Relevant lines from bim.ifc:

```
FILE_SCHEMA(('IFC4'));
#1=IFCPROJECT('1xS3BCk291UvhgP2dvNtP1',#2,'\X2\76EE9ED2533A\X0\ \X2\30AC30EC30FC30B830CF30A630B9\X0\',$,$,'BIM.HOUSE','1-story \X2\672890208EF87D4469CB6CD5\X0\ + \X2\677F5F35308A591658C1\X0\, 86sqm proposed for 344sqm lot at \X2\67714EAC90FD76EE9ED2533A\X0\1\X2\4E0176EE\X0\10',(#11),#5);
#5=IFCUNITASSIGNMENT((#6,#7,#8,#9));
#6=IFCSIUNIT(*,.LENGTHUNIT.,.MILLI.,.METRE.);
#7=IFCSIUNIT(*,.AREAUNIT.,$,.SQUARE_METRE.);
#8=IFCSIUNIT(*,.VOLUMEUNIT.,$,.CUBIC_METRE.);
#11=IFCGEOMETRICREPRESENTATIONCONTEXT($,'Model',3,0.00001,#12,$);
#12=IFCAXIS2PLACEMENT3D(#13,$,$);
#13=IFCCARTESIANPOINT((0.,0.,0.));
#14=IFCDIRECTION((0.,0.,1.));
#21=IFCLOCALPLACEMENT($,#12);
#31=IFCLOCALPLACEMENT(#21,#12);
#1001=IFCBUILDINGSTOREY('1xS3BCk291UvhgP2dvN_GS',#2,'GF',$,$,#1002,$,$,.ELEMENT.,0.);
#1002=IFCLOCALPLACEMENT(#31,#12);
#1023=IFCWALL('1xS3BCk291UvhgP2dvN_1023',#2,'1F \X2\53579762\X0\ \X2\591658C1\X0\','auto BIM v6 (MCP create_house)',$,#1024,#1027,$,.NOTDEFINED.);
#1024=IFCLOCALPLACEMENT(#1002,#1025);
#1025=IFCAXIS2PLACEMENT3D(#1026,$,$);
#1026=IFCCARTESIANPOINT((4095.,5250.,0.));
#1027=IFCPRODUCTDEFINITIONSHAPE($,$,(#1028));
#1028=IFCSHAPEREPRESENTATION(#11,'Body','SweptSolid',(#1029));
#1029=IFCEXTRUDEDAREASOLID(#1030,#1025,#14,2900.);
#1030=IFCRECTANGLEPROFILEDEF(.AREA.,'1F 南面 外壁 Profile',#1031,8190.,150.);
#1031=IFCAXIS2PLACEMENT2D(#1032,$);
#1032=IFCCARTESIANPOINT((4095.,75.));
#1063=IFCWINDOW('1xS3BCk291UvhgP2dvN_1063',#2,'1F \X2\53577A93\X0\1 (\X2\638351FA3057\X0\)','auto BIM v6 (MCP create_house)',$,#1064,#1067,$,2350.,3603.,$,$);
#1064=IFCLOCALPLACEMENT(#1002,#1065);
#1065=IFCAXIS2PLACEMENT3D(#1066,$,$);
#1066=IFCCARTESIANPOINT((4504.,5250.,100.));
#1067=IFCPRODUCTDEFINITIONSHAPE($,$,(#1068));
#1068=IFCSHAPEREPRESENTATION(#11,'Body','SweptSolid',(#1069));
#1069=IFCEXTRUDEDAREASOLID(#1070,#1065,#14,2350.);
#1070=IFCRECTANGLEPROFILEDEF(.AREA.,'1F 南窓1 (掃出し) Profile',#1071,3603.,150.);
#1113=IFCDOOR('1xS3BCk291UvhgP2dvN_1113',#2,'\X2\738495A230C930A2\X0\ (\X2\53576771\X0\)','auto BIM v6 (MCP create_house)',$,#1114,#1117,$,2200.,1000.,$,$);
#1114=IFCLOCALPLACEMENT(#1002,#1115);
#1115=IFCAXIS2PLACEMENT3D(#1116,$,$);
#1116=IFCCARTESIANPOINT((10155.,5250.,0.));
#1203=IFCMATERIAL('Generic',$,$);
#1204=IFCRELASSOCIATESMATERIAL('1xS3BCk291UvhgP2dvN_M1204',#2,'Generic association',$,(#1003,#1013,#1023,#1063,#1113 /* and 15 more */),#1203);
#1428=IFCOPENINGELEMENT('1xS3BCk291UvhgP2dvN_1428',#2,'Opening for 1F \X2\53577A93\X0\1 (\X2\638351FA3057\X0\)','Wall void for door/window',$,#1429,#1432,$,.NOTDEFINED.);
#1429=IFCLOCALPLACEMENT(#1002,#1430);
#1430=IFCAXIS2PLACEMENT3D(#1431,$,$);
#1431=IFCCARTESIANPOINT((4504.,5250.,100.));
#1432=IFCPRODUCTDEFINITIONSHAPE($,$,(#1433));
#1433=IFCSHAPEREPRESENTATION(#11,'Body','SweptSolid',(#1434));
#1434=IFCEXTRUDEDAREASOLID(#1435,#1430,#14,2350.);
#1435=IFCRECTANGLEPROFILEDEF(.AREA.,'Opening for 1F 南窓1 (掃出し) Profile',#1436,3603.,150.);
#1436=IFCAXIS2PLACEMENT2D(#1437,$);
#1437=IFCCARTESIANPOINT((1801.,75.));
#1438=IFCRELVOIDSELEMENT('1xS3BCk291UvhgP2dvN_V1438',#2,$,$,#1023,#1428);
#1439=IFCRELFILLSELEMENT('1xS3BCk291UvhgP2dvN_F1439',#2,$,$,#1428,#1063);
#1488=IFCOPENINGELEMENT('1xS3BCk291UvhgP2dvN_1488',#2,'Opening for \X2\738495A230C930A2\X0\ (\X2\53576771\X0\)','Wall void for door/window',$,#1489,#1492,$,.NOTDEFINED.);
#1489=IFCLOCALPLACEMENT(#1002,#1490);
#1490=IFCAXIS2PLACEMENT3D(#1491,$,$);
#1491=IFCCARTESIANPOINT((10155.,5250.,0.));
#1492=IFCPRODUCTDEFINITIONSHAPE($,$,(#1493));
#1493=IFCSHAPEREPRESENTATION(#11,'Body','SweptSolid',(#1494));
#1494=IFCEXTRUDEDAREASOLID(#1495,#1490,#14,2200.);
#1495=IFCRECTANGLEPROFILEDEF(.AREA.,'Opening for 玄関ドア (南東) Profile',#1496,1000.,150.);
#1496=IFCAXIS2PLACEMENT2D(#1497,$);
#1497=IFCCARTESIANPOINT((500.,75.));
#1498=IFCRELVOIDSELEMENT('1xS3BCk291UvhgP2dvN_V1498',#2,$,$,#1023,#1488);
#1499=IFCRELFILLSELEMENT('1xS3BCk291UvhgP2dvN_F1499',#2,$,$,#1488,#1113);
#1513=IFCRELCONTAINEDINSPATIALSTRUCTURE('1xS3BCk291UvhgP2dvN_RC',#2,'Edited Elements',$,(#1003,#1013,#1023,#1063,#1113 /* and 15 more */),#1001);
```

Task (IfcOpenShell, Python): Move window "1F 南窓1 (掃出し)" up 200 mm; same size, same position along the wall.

```python
import numpy as np
import ifcopenshell
import ifcopenshell.api.geometry
import ifcopenshell.util.placement
import ifcopenshell.util.unit

model = ifcopenshell.open("bim.ifc")
unit_scale = ifcopenshell.util.unit.calculate_unit_scale(model)

window = model.by_guid("1xS3BCk291UvhgP2dvN_1063")
opening = window.FillsVoids[0].RelatingOpeningElement
dz = 0.2 / unit_scale

shift = np.array([0.0, 0.0, dz])
# The window is not placed relative to its opening, so move both.
for product in (opening, window):
    matrix = ifcopenshell.util.placement.get_local_placement(product.ObjectPlacement)
    matrix[:3, 3] += shift
    ifcopenshell.api.geometry.edit_object_placement(model, product=product, matrix=matrix, is_si=False)

print(f"moved by {dz * unit_scale:+.3f} m")

model.write("bim-out.ifc")
```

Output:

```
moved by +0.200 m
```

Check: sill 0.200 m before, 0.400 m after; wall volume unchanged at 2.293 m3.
